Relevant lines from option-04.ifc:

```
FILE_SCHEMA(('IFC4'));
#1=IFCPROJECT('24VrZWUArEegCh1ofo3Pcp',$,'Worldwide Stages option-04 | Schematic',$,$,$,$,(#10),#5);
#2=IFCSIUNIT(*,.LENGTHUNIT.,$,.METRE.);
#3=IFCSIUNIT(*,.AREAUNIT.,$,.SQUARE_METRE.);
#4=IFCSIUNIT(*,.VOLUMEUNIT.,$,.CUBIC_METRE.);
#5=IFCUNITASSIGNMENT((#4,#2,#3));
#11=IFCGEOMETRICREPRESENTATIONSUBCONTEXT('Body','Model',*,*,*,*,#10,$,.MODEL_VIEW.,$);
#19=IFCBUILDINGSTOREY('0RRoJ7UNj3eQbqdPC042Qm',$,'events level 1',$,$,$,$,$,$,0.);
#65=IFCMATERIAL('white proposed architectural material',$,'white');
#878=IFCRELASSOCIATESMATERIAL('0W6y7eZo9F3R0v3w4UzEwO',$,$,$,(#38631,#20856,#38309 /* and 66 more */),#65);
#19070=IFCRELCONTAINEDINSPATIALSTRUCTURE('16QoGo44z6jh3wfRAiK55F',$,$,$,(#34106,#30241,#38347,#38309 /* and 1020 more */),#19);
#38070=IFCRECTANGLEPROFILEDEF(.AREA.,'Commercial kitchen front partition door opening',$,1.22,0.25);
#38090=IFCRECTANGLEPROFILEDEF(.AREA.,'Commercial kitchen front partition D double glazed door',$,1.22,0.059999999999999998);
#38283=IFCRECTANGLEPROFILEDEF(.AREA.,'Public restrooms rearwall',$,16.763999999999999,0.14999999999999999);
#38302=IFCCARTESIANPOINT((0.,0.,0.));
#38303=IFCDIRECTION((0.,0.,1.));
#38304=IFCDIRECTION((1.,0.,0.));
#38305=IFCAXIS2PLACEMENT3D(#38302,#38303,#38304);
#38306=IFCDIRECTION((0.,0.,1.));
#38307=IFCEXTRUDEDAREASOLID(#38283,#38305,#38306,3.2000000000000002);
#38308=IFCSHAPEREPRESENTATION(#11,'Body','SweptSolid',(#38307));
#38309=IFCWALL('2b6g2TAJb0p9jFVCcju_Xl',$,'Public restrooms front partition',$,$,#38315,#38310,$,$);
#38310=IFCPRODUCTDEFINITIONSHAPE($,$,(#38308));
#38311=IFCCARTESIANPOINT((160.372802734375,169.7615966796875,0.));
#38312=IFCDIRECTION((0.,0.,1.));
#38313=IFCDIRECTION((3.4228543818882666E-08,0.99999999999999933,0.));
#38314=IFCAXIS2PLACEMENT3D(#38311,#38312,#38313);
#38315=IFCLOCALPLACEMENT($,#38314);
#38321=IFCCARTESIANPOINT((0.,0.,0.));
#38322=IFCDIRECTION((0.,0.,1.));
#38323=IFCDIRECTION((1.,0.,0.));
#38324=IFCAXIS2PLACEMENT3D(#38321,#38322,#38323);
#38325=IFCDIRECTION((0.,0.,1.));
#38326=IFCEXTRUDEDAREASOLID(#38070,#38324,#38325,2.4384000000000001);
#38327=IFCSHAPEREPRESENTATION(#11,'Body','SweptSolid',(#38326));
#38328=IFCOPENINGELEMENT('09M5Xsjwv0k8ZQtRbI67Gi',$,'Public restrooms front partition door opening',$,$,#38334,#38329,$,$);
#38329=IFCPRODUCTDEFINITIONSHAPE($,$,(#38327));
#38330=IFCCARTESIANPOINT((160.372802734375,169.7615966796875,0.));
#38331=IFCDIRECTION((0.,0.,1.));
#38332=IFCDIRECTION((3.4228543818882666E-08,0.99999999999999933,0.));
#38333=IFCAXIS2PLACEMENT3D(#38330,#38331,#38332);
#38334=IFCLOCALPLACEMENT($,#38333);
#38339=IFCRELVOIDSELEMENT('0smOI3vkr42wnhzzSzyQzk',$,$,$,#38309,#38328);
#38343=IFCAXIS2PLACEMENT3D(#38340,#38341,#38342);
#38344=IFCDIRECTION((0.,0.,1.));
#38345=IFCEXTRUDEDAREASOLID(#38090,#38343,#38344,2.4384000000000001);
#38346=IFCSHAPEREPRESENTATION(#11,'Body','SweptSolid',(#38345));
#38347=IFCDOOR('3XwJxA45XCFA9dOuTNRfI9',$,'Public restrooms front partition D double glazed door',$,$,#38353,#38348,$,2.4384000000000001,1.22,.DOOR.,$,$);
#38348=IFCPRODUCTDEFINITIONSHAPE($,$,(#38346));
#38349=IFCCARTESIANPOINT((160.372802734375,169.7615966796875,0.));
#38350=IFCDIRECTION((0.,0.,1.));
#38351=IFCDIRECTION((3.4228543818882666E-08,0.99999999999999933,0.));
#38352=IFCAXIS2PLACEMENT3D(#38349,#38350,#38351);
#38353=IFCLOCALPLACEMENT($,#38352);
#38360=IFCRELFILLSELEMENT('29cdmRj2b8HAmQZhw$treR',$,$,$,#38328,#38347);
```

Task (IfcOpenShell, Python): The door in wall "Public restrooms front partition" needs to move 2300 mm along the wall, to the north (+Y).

```python
import ifcopenshell
import ifcopenshell.api.geometry
import ifcopenshell.util.placement
import ifcopenshell.util.unit

model = ifcopenshell.open("option-04.ifc")
unit_scale = ifcopenshell.util.unit.calculate_unit_scale(model)

door = model.by_guid("3XwJxA45XCFA9dOuTNRfI9")
opening = door.FillsVoids[0].RelatingOpeningElement
wall = opening.VoidsElements[0].RelatingBuildingElement

wall_matrix = ifcopenshell.util.placement.get_local_placement(wall.ObjectPlacement)
shift = wall_matrix[:3, 0] * 2.3 / unit_scale
before = ifcopenshell.util.placement.get_local_placement(door.ObjectPlacement)[:3, 3].copy()

# The door is not placed relative to its opening, so move both.
for product in (opening, door):
    matrix = ifcopenshell.util.placement.get_local_placement(product.ObjectPlacement)
    matrix[:3, 3] += shift
    ifcopenshell.api.geometry.edit_object_placement(model, product=product, matrix=matrix, is_si=False)

after = ifcopenshell.util.placement.get_local_placement(door.ObjectPlacement)[:3, 3]
print("door moved by", (after - before).round(3) + 0.0)

model.write("option-04_v2.ifc")
```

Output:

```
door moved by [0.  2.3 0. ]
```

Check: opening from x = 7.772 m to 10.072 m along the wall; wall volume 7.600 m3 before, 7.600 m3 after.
